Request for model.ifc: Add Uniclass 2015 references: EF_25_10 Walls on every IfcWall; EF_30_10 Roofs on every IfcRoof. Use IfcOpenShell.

First a look at what the model holds.

```python
import ifcopenshell

model = ifcopenshell.open("model.ifc")
print(model.schema)
print("classifications:", [c.Name for c in model.by_type("IfcClassification")])
for ifc_class in ("IfcDoor", "IfcRoof", "IfcStair", "IfcWall", "IfcWindow"):
    print(ifc_class, len(model.by_type(ifc_class)))
```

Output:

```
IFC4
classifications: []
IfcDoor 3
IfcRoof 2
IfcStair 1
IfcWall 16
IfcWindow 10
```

```python
import ifcopenshell
import ifcopenshell.api.classification

model = ifcopenshell.open("model.ifc")

system = ifcopenshell.api.classification.add_classification(model, classification="Uniclass 2015")

codes = {
    "IfcWall": ("EF_25_10", "Walls"),
    "IfcRoof": ("EF_30_10", "Roofs"),
}
for ifc_class, (code, name) in codes.items():
    products = model.by_type(ifc_class)
    ifcopenshell.api.classification.add_reference(
        model, products=products, classification=system, identification=code, name=name
    )
    print(code, len(products))

model.write("model_updated.ifc")
```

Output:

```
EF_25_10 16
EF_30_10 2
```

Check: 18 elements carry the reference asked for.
